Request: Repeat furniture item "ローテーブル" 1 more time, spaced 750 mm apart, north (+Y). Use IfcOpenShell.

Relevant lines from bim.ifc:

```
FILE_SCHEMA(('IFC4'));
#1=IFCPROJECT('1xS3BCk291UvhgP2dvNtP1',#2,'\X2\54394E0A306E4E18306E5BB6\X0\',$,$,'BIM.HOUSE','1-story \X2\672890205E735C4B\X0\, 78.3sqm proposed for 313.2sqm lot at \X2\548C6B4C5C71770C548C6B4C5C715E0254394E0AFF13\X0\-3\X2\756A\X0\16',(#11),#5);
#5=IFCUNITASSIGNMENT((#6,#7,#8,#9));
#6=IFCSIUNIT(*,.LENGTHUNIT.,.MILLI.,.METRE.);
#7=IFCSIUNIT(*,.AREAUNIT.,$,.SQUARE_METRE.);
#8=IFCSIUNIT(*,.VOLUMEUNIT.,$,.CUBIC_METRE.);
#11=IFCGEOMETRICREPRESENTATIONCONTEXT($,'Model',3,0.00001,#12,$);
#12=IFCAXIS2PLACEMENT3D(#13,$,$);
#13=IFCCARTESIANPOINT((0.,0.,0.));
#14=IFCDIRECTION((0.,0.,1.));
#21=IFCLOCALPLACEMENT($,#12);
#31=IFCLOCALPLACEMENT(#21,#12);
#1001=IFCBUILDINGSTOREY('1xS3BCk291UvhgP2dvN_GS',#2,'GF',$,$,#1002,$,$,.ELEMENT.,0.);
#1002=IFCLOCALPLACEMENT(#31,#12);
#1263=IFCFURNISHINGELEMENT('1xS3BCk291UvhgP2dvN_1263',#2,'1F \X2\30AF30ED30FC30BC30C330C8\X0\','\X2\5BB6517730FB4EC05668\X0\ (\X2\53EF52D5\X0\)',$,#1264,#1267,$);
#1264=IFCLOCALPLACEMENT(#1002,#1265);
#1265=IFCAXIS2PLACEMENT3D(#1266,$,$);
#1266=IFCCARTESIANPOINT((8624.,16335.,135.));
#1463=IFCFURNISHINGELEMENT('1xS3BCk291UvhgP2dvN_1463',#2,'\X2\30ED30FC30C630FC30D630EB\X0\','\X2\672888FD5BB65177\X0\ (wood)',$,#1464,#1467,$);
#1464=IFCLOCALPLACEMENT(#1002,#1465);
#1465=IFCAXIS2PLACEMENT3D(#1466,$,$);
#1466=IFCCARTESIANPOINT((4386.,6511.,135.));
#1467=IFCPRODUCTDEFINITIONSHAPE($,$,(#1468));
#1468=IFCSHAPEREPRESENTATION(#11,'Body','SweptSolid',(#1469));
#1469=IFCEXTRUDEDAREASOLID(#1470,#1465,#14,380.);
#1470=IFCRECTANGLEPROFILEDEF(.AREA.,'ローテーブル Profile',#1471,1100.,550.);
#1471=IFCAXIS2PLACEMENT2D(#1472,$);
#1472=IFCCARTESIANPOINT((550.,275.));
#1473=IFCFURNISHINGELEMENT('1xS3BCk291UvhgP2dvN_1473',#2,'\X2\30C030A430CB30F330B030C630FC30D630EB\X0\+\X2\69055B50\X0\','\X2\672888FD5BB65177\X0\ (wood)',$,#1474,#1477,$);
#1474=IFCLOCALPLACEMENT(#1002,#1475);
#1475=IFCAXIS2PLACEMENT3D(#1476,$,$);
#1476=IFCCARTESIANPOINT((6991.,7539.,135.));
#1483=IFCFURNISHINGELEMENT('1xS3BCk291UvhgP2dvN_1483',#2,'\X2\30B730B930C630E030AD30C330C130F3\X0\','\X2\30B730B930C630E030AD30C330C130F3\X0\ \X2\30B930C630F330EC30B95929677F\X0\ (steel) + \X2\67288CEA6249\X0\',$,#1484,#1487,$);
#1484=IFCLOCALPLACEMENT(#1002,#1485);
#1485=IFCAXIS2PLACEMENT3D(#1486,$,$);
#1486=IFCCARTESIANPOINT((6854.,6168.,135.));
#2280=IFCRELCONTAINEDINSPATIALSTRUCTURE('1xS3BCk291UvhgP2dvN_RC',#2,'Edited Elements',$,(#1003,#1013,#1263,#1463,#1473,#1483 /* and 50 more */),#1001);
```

```python
import numpy as np
import ifcopenshell
import ifcopenshell.api.geometry
import ifcopenshell.api.root
import ifcopenshell.util.element
import ifcopenshell.util.placement
import ifcopenshell.util.unit

model = ifcopenshell.open("bim.ifc")
unit_scale = ifcopenshell.util.unit.calculate_unit_scale(model)


def reuse_history(source, copy):
    """copy_class also copies each property set's owner history, people and application; keep the originals."""
    for rel in copy.IsDefinedBy:
        if rel.is_a("IfcRelDefinesByProperties") and (history := rel.RelatingPropertyDefinition.OwnerHistory):
            rel.RelatingPropertyDefinition.OwnerHistory = source.OwnerHistory
            ifcopenshell.util.element.remove_deep2(model, history)


source = model.by_guid("1xS3BCk291UvhgP2dvN_1463")
base = ifcopenshell.util.placement.get_local_placement(source.ObjectPlacement)
step = np.array([0.0, 1.0, 0.0]) * 0.75 / unit_scale

for i in range(1, 2):
    copy = ifcopenshell.api.root.copy_class(model, product=source)
    copy.Representation = ifcopenshell.util.element.copy_deep(
        model, source.Representation, exclude=["IfcGeometricRepresentationContext", "IfcRepresentationMap"]
    )
    reuse_history(source, copy)
    matrix = base.copy()
    matrix[:3, 3] += i * step
    print("added at", matrix[:3, 3].round(3) + 0.0)
    ifcopenshell.api.geometry.edit_object_placement(model, product=copy, matrix=matrix, is_si=False)

model.write("bim_edited.ifc")
```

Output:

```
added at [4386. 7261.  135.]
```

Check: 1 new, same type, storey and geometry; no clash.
